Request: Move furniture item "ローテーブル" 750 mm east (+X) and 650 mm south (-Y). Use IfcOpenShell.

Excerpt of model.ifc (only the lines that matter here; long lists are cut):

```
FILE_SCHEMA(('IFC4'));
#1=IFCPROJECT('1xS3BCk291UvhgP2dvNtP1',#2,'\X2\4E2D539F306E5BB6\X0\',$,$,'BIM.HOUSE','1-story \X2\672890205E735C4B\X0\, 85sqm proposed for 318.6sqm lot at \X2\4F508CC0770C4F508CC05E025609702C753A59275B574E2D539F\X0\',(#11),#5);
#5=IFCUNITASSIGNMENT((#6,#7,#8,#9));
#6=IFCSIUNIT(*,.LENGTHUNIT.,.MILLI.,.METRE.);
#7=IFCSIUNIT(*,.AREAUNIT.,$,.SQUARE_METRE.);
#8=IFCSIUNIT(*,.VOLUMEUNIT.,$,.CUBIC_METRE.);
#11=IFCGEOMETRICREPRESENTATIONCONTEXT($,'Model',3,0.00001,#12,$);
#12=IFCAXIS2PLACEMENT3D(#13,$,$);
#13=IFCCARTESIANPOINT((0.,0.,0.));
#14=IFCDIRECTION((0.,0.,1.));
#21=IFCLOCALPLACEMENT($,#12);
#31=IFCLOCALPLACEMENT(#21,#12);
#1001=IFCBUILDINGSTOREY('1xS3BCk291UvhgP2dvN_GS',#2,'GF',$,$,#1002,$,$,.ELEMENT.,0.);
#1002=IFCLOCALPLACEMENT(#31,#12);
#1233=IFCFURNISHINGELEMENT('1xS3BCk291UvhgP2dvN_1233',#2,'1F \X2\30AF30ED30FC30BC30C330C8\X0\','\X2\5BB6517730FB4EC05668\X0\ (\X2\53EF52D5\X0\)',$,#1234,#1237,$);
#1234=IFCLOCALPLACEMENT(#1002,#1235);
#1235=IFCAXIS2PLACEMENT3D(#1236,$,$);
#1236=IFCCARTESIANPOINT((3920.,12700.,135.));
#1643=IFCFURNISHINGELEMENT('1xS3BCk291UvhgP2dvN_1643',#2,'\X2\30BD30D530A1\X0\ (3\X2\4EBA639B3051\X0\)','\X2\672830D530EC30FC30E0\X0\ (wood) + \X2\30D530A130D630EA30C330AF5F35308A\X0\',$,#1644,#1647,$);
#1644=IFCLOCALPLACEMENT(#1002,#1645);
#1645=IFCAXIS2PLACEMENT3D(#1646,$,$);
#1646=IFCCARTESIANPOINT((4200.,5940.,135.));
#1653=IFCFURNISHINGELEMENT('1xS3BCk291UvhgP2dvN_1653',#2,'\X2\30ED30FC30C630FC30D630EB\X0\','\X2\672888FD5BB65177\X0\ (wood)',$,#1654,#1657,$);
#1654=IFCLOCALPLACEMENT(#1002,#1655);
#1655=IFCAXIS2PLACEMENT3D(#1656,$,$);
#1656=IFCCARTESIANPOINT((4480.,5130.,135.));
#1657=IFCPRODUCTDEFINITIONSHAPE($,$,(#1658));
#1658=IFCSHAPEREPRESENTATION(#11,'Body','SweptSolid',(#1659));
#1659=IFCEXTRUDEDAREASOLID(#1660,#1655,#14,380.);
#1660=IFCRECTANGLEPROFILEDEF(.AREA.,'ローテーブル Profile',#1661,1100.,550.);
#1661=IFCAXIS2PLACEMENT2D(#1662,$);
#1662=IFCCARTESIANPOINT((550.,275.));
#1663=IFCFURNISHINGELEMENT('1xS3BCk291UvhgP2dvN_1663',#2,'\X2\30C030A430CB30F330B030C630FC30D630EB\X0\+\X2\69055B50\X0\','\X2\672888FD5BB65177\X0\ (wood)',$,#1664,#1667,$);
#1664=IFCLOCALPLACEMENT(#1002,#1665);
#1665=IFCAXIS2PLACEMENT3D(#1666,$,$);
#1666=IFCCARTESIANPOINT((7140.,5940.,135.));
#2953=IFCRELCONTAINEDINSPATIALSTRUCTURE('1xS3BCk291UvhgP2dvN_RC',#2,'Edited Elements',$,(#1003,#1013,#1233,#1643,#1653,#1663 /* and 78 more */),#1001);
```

```python
import ifcopenshell
import ifcopenshell.api.geometry
import ifcopenshell.util.placement

model = ifcopenshell.open("model.ifc")

item = model.by_guid("1xS3BCk291UvhgP2dvN_1653")
matrix = ifcopenshell.util.placement.get_local_placement(item.ObjectPlacement)
matrix[0, 3] += 750.0
matrix[1, 3] -= 650.0
ifcopenshell.api.geometry.edit_object_placement(model, product=item, matrix=matrix, is_si=False)

print(ifcopenshell.util.placement.get_local_placement(item.ObjectPlacement).round(3) + 0.0)

model.write("model_v2.ifc")
```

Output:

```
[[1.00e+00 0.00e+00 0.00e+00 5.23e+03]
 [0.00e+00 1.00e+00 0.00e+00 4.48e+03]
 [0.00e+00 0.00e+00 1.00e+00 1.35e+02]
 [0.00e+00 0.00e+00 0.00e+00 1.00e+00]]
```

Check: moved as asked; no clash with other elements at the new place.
